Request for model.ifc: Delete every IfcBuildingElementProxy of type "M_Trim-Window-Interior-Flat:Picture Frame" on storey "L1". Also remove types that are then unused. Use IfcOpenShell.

First a look at what the model holds.

```python
import ifcopenshell
import ifcopenshell.util.element

model = ifcopenshell.open("model.ifc")
print(model.schema)
storey = next(s for s in model.by_type("IfcBuildingStorey") if s.Name == "L1")
proxies = [e for e in ifcopenshell.util.element.get_decomposition(storey) if e.is_a("IfcBuildingElementProxy")]
seen = {}
for e in proxies:
    element_type = ifcopenshell.util.element.get_type(e)
    name = element_type.Name if element_type not in (None, e) else None
    seen[name] = seen.get(name, 0) + 1
for name, count in sorted(seen.items(), key=str):
    print(count, "x", name)
```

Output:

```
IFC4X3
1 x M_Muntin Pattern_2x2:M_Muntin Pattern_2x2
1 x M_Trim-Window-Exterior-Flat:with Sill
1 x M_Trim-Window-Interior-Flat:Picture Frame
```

```python
import ifcopenshell
import ifcopenshell.api.root
import ifcopenshell.util.element

model = ifcopenshell.open("model.ifc")

storey = next(s for s in model.by_type("IfcBuildingStorey") if s.Name == "L1")
proxies = [e for e in ifcopenshell.util.element.get_decomposition(storey) if e.is_a("IfcBuildingElementProxy")]
targets = [e for e in proxies if (t := ifcopenshell.util.element.get_type(e)) not in (None, e) and t.Name == "M_Trim-Window-Interior-Flat:Picture Frame"]
types = {ifcopenshell.util.element.get_type(e) for e in targets} - {None, *targets}

for e in targets:
    ifcopenshell.api.root.remove_product(model, product=e)
print(len(targets), "removed")

unused = [t for t in types if not ifcopenshell.util.element.get_types(t)]
for t in unused:
    ifcopenshell.api.root.remove_product(model, product=t)
print(len(unused), "unused types removed")

model.write("model_edited.ifc")
```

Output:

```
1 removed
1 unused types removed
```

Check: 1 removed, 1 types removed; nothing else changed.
